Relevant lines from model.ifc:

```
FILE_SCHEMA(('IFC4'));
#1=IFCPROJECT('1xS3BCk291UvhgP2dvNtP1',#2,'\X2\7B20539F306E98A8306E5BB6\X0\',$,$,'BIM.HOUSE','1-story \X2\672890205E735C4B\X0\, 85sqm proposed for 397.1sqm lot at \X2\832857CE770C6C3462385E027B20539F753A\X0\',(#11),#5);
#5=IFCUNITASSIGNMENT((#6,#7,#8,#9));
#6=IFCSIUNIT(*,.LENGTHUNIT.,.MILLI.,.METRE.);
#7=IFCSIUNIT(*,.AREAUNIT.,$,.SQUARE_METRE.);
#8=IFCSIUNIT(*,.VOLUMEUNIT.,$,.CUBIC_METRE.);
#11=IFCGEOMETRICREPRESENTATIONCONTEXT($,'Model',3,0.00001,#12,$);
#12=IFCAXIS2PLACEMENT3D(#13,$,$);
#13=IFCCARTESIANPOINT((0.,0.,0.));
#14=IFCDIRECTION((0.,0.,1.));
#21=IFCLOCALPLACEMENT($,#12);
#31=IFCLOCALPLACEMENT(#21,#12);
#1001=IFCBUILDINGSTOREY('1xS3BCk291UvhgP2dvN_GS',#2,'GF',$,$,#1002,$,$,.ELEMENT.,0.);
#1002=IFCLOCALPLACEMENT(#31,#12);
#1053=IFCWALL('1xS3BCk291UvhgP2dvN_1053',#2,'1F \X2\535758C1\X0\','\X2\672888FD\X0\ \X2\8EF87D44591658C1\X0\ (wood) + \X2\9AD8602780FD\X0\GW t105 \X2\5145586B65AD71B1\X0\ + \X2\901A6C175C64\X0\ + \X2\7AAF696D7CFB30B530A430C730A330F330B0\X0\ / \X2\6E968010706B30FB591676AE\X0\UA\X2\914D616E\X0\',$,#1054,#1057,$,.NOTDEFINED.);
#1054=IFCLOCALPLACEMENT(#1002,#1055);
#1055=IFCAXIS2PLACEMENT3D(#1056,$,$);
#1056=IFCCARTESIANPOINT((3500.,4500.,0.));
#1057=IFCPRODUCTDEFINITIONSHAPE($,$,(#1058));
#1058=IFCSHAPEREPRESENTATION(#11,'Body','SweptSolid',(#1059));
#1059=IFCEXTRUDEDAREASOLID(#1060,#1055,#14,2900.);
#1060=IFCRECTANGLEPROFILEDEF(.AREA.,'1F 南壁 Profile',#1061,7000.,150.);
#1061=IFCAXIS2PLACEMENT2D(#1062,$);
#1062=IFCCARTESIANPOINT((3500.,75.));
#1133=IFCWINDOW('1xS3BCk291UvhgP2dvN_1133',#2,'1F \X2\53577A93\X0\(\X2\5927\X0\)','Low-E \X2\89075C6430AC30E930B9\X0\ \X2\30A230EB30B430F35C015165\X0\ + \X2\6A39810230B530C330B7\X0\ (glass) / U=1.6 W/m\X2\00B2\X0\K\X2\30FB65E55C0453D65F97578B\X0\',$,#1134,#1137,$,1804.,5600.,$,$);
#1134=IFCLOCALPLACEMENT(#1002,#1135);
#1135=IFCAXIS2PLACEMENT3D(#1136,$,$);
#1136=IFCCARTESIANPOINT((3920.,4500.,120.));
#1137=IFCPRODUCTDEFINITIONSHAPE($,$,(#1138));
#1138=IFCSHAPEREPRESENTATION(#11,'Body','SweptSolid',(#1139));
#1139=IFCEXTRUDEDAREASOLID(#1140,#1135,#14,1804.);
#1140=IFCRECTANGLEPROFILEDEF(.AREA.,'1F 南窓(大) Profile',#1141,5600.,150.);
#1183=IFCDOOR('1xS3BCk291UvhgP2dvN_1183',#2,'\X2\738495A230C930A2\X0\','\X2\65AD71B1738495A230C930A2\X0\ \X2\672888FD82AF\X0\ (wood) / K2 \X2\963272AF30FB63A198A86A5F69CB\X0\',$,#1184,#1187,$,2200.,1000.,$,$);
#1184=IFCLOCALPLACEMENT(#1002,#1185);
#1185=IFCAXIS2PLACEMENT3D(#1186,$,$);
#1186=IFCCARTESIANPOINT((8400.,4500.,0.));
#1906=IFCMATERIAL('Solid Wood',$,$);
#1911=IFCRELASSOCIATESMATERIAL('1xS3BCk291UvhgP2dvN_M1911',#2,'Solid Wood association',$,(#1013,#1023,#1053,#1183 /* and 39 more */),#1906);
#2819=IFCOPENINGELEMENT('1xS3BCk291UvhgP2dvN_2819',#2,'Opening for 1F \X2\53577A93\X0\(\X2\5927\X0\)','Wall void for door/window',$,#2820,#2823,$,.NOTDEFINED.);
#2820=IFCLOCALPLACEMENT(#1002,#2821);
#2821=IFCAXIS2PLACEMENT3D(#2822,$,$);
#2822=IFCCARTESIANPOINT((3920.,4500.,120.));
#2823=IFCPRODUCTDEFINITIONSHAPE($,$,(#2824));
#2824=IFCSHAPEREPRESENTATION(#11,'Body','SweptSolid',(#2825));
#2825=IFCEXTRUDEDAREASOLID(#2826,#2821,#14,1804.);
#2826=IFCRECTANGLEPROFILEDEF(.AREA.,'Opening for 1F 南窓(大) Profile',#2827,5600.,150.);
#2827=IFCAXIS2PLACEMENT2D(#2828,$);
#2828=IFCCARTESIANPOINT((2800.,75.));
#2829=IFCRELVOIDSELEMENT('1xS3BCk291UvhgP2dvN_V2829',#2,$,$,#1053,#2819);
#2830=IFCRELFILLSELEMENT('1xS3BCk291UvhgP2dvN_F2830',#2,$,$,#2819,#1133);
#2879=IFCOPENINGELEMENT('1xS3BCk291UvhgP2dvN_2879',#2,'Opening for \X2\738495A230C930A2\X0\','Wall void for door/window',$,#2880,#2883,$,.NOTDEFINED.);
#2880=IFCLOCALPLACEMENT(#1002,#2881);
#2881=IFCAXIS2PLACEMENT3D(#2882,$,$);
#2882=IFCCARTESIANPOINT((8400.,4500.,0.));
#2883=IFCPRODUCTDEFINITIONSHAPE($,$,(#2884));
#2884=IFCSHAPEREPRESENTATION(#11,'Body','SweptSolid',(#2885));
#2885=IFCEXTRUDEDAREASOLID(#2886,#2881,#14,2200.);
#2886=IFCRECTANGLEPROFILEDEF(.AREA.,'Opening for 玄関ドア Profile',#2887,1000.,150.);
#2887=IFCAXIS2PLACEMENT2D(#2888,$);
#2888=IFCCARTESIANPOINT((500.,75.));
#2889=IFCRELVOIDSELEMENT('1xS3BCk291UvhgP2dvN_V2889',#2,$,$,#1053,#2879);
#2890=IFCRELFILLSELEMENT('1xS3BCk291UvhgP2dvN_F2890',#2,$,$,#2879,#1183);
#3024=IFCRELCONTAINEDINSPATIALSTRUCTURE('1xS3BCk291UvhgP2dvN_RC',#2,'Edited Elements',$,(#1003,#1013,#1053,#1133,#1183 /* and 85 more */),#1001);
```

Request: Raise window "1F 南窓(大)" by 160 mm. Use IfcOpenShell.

```python
import numpy as np
import ifcopenshell
import ifcopenshell.api.geometry
import ifcopenshell.util.placement
import ifcopenshell.util.unit

model = ifcopenshell.open("model.ifc")
unit_scale = ifcopenshell.util.unit.calculate_unit_scale(model)

window = model.by_id(1133)
opening = window.FillsVoids[0].RelatingOpeningElement
dz = 0.16 / unit_scale

shift = np.array([0.0, 0.0, dz])
# The window is not placed relative to its opening, so move both.
for product in (opening, window):
    matrix = ifcopenshell.util.placement.get_local_placement(product.ObjectPlacement)
    matrix[:3, 3] += shift
    ifcopenshell.api.geometry.edit_object_placement(model, product=product, matrix=matrix, is_si=False)

print(f"moved by {dz * unit_scale:+.3f} m")

model.write("model_updated.ifc")
```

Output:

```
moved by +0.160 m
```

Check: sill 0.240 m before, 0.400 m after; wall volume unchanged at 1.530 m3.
